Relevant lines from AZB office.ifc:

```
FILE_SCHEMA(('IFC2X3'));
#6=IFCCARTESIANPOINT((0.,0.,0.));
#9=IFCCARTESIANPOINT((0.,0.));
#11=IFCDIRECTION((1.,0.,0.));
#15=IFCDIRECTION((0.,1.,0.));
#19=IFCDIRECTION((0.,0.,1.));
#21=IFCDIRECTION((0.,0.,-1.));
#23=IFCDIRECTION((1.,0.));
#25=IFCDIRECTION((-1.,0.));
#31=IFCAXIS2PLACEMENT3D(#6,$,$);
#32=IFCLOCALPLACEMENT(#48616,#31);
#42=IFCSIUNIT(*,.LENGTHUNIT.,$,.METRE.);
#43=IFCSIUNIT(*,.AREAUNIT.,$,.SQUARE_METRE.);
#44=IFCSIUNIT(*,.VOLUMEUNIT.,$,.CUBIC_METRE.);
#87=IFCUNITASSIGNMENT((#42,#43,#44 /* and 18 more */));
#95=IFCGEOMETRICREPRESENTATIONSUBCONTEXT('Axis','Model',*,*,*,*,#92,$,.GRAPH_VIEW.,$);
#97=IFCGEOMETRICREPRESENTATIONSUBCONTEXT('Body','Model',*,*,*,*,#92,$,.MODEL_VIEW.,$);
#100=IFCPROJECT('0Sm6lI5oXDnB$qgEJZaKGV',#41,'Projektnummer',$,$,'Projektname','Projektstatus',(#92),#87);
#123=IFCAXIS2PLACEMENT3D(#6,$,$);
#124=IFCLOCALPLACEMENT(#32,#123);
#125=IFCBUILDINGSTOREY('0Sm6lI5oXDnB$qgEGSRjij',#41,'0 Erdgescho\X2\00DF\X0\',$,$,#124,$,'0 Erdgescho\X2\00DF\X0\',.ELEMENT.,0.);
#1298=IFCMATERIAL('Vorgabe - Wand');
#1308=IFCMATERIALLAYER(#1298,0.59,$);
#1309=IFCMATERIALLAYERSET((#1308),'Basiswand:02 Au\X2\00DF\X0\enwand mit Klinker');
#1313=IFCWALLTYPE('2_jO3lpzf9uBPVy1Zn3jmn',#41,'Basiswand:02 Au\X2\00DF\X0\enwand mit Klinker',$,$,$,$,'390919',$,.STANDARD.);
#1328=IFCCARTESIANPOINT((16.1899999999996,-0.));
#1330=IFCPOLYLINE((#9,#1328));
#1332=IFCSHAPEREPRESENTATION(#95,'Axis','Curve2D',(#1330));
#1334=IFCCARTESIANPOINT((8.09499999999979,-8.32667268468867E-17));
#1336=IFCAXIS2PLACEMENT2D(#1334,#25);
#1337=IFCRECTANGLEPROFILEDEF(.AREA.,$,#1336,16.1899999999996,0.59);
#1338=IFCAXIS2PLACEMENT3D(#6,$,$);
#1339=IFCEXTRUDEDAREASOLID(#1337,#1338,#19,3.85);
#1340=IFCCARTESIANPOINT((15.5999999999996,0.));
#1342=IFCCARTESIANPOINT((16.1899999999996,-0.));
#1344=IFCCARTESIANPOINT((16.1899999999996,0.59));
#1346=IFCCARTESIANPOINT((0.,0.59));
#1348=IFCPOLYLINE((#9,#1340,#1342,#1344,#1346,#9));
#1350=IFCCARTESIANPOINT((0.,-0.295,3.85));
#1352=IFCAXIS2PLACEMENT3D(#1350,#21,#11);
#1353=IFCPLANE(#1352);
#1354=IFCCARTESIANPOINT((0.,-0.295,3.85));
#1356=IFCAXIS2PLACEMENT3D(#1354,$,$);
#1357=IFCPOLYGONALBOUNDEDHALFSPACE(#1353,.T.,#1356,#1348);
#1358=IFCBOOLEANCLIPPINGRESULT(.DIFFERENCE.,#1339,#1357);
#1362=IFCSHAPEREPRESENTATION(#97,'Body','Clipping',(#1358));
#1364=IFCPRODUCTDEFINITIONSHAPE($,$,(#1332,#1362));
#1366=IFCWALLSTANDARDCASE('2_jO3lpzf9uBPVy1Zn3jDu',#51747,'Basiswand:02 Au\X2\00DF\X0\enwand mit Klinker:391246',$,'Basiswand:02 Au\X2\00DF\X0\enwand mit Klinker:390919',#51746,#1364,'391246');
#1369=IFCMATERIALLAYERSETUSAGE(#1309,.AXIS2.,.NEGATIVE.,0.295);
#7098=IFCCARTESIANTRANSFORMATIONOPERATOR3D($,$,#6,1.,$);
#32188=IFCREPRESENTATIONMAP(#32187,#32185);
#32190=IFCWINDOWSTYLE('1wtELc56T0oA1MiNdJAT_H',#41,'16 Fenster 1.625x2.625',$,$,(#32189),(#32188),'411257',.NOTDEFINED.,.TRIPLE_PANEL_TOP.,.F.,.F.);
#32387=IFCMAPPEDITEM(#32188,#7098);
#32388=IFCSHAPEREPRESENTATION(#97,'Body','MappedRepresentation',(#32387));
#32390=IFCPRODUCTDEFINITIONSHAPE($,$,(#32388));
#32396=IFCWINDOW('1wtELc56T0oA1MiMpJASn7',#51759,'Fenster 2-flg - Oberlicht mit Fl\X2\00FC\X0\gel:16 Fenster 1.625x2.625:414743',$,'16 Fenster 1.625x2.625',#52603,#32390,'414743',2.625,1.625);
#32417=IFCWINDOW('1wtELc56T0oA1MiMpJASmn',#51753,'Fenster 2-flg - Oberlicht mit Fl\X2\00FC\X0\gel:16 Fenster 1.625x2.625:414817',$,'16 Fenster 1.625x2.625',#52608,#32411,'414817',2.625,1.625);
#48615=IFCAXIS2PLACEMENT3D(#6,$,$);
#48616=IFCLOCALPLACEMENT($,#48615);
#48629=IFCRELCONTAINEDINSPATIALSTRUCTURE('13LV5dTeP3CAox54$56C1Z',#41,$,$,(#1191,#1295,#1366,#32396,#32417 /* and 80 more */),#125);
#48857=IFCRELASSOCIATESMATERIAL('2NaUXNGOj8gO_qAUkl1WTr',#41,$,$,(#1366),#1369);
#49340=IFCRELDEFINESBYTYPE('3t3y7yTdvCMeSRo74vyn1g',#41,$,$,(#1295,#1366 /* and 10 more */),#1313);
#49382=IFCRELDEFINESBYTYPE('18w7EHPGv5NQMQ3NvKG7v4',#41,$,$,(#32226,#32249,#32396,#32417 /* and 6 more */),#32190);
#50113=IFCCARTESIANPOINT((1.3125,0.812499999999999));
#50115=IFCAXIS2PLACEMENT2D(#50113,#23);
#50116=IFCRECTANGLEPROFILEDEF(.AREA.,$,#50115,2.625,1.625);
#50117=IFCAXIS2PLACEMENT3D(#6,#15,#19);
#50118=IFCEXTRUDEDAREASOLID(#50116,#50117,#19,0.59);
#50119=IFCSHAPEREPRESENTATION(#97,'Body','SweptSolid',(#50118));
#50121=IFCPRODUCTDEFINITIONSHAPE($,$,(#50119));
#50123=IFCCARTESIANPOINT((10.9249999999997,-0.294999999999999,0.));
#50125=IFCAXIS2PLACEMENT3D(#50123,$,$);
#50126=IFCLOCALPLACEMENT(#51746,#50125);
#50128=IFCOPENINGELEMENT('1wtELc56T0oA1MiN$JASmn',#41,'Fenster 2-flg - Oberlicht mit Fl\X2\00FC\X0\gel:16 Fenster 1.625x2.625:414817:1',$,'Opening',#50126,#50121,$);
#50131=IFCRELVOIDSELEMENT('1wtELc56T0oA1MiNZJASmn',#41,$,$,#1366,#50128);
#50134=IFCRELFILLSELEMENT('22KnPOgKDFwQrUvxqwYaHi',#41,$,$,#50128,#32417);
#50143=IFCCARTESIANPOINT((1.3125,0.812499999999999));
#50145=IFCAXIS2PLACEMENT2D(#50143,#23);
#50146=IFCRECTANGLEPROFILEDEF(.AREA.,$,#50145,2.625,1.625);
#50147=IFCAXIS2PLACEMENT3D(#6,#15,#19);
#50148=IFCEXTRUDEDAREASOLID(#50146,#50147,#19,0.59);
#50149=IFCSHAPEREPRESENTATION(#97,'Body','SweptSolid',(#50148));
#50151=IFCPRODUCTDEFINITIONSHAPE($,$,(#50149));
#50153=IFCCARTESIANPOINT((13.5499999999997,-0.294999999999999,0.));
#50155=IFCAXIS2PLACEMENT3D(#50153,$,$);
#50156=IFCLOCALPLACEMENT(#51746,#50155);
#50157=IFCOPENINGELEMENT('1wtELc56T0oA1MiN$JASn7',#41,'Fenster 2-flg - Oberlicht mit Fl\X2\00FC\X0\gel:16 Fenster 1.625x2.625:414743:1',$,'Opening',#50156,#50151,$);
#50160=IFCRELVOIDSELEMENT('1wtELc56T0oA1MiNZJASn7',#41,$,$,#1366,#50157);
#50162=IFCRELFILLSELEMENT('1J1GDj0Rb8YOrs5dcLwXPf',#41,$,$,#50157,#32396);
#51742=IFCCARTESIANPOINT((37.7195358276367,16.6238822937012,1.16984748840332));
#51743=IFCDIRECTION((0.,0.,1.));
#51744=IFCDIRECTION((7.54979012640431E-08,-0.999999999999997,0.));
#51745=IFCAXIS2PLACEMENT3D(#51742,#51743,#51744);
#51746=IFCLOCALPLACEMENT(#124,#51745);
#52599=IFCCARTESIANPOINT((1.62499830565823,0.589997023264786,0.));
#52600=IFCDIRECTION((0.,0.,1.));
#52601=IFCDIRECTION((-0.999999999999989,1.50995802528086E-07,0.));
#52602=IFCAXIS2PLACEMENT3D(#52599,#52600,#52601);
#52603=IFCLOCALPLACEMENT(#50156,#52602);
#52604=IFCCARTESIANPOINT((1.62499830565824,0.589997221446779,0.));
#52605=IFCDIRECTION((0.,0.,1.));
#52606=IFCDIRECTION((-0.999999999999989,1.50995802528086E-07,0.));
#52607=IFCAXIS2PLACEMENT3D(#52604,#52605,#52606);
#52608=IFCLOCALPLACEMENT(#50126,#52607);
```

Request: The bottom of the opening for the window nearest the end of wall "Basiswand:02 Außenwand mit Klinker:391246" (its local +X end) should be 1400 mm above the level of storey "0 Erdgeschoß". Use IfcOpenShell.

```python
import numpy as np
import ifcopenshell
import ifcopenshell.api.geometry
import ifcopenshell.geom
import ifcopenshell.util.element
import ifcopenshell.util.placement
import ifcopenshell.util.shape
import ifcopenshell.util.unit

model = ifcopenshell.open("AZB office.ifc")
unit_scale = ifcopenshell.util.unit.calculate_unit_scale(model)

window = model.by_id(32396)
opening = window.FillsVoids[0].RelatingOpeningElement
storey = ifcopenshell.util.element.get_container(window, ifc_class="IfcBuildingStorey")
level = ifcopenshell.util.placement.get_local_placement(storey.ObjectPlacement)[2, 3]

# The opening's origin need not be at the sill, so measure its lowest point.
shape = ifcopenshell.geom.create_shape(ifcopenshell.geom.settings(), opening)
bottom = ifcopenshell.util.shape.get_shape_bottom_elevation(shape, shape.geometry) / unit_scale
dz = level + 1.4 / unit_scale - bottom

shift = np.array([0.0, 0.0, dz])
# The window is placed relative to its opening, so it follows when the opening moves.
matrix = ifcopenshell.util.placement.get_local_placement(opening.ObjectPlacement)
matrix[:3, 3] += shift
ifcopenshell.api.geometry.edit_object_placement(
    model, product=opening, matrix=matrix, is_si=False, should_transform_children=True
)

print(f"moved by {dz * unit_scale:+.3f} m")

model.write("AZB office_v2.ifc")
```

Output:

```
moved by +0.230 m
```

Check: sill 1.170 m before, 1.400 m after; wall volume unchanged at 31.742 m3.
